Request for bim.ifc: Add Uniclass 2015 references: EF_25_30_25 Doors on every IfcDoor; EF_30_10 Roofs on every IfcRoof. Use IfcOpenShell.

First a look at what the model holds.

```python
import ifcopenshell

model = ifcopenshell.open("bim.ifc")
print(model.schema)
print("classifications:", [c.Name for c in model.by_type("IfcClassification")])
for ifc_class in ("IfcDoor", "IfcRoof", "IfcStair", "IfcWall", "IfcWindow"):
    print(ifc_class, len(model.by_type(ifc_class)))
```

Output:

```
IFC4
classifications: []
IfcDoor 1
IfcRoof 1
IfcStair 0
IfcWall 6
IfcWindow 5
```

```python
import ifcopenshell
import ifcopenshell.api.classification

model = ifcopenshell.open("bim.ifc")

system = ifcopenshell.api.classification.add_classification(model, classification="Uniclass 2015")

codes = {
    "IfcDoor": ("EF_25_30_25", "Doors"),
    "IfcRoof": ("EF_30_10", "Roofs"),
}
for ifc_class, (code, name) in codes.items():
    products = model.by_type(ifc_class)
    ifcopenshell.api.classification.add_reference(
        model, products=products, classification=system, identification=code, name=name
    )
    print(code, len(products))

model.write("bim_rev.ifc")
```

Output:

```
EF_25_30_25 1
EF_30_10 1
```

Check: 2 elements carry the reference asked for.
